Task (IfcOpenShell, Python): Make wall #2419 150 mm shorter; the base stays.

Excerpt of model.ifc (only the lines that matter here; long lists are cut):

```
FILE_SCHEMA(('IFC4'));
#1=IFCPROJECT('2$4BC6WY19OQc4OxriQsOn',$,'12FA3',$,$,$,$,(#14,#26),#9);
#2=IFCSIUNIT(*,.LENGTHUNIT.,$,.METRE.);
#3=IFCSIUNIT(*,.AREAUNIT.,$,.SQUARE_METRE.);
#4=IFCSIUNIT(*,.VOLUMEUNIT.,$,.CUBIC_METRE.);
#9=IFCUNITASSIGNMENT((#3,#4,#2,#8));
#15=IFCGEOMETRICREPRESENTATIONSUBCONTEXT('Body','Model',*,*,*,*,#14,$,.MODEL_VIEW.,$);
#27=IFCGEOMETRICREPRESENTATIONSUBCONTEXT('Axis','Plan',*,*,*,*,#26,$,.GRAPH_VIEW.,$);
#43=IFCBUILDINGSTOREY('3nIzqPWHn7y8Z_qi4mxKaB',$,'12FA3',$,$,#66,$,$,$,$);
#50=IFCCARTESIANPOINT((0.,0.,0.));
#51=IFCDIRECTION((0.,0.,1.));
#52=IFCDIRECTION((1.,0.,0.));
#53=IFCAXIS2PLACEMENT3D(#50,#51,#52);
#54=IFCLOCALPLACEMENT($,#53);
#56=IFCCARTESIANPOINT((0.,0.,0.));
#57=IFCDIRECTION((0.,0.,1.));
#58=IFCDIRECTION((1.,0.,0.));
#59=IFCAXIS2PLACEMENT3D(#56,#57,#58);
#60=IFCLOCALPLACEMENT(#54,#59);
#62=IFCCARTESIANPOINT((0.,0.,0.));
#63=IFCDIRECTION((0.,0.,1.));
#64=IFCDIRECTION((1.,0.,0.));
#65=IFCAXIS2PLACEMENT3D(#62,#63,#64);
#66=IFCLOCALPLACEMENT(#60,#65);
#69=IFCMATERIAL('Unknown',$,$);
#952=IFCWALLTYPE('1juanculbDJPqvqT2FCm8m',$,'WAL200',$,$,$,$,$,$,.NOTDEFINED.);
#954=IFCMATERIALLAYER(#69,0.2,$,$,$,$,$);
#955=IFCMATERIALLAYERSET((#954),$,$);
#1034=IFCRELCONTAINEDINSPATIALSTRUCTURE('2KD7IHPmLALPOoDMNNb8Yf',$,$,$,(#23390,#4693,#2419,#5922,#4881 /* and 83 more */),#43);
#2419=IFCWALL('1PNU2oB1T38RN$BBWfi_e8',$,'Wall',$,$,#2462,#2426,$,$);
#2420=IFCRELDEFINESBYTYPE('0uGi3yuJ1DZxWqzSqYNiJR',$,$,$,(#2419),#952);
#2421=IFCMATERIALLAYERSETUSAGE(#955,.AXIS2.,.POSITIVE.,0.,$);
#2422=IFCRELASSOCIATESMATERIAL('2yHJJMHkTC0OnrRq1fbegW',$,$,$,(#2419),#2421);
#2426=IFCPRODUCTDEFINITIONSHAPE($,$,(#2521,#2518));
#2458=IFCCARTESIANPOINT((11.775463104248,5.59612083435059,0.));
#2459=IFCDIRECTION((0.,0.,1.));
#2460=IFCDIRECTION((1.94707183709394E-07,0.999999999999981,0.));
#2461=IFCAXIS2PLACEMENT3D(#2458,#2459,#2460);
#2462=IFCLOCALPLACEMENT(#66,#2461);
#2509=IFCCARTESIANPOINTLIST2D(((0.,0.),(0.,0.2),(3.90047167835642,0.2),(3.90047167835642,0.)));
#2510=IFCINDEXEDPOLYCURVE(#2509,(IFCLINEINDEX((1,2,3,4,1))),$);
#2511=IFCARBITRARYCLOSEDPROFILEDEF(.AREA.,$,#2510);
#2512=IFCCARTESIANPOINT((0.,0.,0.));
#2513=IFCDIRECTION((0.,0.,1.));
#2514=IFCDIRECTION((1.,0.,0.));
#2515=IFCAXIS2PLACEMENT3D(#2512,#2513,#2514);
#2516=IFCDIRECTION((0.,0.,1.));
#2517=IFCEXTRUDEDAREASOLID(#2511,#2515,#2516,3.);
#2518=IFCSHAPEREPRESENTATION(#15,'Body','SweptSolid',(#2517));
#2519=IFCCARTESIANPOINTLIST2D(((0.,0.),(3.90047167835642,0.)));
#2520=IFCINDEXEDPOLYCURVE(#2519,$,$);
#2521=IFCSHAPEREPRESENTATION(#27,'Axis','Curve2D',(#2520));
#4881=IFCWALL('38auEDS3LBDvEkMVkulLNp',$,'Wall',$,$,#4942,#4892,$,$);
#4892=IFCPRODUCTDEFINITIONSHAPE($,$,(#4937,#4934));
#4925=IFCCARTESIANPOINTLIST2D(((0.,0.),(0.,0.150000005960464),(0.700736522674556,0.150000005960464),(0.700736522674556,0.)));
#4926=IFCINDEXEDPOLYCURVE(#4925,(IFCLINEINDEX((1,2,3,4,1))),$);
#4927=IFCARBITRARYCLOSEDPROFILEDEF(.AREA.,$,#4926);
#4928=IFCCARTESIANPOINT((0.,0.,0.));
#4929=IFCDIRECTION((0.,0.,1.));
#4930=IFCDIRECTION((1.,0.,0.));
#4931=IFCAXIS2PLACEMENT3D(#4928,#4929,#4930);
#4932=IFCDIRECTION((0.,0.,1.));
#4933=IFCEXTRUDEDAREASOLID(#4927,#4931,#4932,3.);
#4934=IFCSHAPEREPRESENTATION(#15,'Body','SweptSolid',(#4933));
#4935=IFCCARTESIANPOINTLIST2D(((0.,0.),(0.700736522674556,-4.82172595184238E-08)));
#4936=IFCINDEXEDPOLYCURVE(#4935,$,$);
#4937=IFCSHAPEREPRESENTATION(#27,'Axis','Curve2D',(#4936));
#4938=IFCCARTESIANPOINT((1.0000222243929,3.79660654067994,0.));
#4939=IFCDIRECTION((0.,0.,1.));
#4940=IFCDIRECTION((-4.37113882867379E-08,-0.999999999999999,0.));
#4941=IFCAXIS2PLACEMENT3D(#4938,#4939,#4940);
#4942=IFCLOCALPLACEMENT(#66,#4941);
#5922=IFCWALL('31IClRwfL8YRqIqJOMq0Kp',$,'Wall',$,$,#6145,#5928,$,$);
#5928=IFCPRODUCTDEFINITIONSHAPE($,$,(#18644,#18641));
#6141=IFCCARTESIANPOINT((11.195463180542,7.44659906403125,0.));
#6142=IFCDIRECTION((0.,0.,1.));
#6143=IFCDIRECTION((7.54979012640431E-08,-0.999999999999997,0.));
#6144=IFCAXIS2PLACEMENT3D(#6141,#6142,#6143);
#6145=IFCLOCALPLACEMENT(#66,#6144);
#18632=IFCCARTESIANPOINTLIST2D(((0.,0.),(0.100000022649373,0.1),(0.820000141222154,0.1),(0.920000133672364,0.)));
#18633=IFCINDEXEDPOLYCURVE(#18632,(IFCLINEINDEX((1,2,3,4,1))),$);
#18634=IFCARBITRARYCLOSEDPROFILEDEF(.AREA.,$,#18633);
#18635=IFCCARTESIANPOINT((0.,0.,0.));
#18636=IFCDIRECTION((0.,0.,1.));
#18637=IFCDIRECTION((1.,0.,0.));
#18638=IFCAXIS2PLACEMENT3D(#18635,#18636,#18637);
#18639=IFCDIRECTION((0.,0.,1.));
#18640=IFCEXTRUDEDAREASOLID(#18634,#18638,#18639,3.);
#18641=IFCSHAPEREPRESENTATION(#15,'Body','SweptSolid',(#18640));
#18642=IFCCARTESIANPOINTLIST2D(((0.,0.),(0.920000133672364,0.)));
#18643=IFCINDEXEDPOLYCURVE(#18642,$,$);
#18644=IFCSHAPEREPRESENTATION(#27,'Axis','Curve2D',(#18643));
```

```python
import ifcopenshell
import ifcopenshell.geom
import ifcopenshell.util.representation
import ifcopenshell.util.shape

model = ifcopenshell.open("model.ifc")
settings = ifcopenshell.geom.settings()


def volume(element):
    """Net volume in cubic metres, openings subtracted."""
    shape = ifcopenshell.geom.create_shape(settings, element)
    return ifcopenshell.util.shape.get_volume(shape.geometry)


wall = model.by_id(2419)
before = volume(wall)

body = ifcopenshell.util.representation.get_representation(wall, "Model", "Body")
solid = body.Items[0]
old_height = solid.Depth
solid.Depth -= 0.15
after = volume(wall)

print(f"height {old_height:g} -> {solid.Depth:g}, volume {before:.3f} -> {after:.3f} m3")

model.write("model_updated.ifc")
```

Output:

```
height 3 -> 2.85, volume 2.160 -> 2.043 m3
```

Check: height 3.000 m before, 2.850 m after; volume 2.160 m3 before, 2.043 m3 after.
